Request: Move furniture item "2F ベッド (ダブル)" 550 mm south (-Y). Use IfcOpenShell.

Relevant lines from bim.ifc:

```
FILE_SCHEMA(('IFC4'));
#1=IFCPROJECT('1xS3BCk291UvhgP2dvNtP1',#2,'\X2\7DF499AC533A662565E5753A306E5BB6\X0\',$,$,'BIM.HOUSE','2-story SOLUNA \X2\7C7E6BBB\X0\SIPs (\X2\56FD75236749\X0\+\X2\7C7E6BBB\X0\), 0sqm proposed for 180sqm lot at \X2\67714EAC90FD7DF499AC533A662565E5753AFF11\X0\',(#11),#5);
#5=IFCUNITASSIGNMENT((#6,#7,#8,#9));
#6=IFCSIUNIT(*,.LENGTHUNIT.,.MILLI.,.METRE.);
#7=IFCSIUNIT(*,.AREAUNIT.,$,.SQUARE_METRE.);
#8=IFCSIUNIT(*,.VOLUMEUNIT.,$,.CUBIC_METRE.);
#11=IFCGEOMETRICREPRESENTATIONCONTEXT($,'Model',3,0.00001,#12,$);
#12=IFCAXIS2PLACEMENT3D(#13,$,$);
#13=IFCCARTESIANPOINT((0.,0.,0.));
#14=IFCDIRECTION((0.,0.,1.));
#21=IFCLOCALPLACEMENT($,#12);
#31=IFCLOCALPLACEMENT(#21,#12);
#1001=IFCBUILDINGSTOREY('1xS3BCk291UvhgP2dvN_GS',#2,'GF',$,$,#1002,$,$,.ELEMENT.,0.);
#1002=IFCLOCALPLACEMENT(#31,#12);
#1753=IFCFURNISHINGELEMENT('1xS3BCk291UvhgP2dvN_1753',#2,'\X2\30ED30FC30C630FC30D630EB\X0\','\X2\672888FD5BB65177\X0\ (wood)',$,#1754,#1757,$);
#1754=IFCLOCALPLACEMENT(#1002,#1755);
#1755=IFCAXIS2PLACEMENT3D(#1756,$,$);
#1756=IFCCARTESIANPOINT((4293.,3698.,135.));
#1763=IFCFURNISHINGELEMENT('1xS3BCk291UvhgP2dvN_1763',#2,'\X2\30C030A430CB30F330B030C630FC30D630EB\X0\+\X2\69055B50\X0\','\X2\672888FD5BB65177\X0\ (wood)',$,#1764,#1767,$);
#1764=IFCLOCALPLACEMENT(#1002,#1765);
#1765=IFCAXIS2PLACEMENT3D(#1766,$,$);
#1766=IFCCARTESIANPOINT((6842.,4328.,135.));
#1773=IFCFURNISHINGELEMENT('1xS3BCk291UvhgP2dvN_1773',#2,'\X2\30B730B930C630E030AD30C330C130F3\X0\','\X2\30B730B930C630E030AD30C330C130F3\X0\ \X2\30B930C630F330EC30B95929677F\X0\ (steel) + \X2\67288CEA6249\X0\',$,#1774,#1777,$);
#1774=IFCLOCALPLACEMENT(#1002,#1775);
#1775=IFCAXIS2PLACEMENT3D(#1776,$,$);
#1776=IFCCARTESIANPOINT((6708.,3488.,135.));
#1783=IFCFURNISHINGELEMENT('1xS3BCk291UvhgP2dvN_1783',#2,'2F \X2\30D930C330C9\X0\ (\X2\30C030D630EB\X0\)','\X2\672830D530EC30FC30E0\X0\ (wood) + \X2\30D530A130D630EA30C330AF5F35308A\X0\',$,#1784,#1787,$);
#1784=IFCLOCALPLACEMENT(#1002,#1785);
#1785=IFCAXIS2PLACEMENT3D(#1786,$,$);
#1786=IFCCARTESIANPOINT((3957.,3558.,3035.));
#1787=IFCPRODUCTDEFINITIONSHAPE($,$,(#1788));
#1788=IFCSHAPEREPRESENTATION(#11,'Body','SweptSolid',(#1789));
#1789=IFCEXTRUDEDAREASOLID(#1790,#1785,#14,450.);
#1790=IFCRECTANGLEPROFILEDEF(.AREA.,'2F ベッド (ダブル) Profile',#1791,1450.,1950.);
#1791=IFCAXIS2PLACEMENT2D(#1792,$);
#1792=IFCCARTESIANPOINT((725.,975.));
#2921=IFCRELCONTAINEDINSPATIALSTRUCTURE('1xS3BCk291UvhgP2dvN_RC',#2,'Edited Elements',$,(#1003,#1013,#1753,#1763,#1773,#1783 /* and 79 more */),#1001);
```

```python
import ifcopenshell
import ifcopenshell.api.geometry
import ifcopenshell.util.placement

model = ifcopenshell.open("bim.ifc")

item = model.by_guid("1xS3BCk291UvhgP2dvN_1783")
matrix = ifcopenshell.util.placement.get_local_placement(item.ObjectPlacement)
matrix[1, 3] -= 550.0
ifcopenshell.api.geometry.edit_object_placement(model, product=item, matrix=matrix, is_si=False)

print(ifcopenshell.util.placement.get_local_placement(item.ObjectPlacement).round(3) + 0.0)

model.write("bim-out.ifc")
```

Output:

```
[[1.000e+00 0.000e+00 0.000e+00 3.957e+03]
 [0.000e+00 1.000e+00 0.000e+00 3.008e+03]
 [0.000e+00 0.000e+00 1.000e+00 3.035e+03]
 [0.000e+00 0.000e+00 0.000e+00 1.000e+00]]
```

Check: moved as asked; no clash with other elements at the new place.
